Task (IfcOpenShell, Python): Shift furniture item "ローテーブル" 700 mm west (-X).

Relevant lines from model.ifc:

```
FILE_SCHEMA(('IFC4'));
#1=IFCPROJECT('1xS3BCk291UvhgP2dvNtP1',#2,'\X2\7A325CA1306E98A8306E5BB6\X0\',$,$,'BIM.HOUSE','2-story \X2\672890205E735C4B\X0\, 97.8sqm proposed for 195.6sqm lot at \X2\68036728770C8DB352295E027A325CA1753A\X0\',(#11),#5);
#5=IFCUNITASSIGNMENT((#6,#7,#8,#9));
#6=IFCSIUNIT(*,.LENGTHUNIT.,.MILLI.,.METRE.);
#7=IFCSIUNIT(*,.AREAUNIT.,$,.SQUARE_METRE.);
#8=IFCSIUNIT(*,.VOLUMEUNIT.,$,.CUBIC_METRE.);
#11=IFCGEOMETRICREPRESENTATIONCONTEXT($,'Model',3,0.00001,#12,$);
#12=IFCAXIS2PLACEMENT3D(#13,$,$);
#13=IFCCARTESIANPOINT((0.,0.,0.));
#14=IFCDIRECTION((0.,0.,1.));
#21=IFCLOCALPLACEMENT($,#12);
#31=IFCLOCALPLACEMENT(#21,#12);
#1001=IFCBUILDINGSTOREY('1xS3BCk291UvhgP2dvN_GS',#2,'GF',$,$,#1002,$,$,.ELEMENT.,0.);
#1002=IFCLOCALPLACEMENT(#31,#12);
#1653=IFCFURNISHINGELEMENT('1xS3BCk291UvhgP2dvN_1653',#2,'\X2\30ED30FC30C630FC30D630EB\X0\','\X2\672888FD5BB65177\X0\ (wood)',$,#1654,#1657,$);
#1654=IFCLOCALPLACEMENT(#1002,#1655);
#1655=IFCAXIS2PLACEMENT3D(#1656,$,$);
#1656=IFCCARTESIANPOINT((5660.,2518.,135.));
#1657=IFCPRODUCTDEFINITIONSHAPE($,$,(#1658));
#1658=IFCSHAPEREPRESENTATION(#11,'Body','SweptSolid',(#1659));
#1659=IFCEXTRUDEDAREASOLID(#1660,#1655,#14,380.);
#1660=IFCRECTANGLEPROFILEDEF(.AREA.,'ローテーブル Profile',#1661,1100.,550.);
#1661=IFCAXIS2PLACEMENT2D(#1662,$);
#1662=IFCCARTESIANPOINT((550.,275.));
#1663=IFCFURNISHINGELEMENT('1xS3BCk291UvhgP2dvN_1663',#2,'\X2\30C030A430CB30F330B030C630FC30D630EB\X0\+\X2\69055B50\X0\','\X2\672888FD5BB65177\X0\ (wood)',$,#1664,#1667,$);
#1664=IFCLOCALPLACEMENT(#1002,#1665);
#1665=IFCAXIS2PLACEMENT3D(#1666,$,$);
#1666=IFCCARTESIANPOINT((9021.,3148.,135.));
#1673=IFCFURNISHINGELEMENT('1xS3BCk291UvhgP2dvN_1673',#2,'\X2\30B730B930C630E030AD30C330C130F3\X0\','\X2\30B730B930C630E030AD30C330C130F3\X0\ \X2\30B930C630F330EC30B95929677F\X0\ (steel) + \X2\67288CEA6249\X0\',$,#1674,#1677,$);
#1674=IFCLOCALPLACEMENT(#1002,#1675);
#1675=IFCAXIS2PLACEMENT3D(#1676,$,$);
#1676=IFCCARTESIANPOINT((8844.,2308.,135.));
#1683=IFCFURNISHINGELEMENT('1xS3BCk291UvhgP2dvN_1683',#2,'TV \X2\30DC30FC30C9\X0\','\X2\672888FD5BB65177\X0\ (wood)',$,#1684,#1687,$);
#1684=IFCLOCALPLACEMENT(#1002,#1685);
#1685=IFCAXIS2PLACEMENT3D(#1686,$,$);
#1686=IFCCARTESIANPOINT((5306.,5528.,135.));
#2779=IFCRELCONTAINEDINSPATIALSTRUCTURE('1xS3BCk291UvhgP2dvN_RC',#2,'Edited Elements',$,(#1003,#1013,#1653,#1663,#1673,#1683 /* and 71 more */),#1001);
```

```python
import ifcopenshell
import ifcopenshell.api.geometry
import ifcopenshell.util.placement
import ifcopenshell.util.unit

model = ifcopenshell.open("model.ifc")
unit_scale = ifcopenshell.util.unit.calculate_unit_scale(model)

item = model.by_guid("1xS3BCk291UvhgP2dvN_1653")
matrix = ifcopenshell.util.placement.get_local_placement(item.ObjectPlacement)
matrix[0, 3] -= 0.7 / unit_scale
ifcopenshell.api.geometry.edit_object_placement(model, product=item, matrix=matrix, is_si=False)

print(ifcopenshell.util.placement.get_local_placement(item.ObjectPlacement).round(3) + 0.0)

model.write("model_v2.ifc")
```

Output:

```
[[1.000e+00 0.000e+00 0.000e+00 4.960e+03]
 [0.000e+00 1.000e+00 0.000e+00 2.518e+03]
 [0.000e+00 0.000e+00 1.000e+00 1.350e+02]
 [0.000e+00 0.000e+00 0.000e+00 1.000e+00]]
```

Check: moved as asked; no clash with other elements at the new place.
